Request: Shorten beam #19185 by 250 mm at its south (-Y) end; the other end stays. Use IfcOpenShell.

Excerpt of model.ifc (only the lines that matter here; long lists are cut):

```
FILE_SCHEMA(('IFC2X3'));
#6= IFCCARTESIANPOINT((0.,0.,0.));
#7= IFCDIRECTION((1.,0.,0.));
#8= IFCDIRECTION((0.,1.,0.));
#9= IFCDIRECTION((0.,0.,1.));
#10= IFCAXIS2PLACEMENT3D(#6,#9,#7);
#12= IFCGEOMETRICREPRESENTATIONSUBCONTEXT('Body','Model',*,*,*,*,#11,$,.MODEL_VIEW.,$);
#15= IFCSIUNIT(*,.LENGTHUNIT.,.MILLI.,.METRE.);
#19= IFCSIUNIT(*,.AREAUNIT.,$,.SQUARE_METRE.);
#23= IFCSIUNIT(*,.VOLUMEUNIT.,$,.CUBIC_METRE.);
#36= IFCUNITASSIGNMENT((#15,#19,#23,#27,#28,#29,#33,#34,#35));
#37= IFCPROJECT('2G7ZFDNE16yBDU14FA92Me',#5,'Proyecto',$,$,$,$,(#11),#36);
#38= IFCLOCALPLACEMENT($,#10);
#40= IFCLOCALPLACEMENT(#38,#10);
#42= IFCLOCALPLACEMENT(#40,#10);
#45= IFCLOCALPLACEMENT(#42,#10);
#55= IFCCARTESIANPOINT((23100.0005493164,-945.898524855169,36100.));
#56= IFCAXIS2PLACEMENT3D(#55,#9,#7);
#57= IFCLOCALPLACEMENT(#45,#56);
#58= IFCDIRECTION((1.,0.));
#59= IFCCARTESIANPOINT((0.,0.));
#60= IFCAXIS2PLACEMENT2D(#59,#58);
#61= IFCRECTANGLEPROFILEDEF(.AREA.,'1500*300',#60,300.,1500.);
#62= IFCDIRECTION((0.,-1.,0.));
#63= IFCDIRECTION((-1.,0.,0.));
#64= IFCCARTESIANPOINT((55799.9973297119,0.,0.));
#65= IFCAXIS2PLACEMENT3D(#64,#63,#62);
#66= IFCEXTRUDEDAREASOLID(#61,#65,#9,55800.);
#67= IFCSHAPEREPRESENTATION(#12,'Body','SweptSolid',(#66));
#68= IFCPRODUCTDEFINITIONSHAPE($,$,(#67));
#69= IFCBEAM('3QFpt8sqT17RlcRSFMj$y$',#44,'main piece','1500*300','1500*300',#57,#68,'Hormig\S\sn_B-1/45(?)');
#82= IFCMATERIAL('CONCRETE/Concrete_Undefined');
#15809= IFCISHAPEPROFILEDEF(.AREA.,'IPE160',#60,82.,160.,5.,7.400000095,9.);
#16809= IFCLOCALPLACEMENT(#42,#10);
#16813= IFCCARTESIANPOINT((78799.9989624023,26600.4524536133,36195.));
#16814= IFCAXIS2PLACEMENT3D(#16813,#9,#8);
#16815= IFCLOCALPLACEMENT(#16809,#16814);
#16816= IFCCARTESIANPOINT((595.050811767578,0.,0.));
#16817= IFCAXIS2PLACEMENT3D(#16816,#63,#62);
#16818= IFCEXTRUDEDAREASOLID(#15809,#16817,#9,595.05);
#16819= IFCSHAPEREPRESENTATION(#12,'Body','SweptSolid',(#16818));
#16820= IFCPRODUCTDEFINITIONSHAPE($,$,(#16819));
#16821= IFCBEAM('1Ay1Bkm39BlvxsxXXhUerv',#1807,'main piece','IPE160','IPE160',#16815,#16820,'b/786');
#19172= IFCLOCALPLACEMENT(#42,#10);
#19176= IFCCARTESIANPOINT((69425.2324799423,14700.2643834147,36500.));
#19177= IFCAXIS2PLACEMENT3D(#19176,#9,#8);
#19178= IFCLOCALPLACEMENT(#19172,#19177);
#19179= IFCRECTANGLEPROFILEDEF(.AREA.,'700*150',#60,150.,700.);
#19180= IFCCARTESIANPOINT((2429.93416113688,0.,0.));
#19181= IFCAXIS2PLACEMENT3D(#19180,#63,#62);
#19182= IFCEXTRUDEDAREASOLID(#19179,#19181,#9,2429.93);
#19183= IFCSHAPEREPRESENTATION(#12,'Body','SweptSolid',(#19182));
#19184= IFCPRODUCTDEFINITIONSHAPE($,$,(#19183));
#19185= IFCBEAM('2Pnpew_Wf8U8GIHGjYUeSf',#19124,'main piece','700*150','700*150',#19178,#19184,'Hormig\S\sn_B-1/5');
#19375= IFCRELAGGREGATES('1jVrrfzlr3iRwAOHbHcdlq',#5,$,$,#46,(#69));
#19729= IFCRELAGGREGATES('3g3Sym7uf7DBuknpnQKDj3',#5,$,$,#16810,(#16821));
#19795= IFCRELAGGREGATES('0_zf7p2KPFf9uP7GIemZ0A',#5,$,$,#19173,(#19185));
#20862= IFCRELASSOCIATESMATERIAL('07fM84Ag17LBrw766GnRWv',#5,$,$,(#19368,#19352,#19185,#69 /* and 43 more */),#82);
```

```python
import ifcopenshell
import ifcopenshell.util.representation
import ifcopenshell.util.unit

model = ifcopenshell.open("model.ifc")
unit_scale = ifcopenshell.util.unit.calculate_unit_scale(model)

member = model.by_guid("2Pnpew_Wf8U8GIHGjYUeSf")
change = -0.25 / unit_scale

# The extrusion runs towards the end named, so only its depth changes.
body = ifcopenshell.util.representation.get_representation(member, "Model", "Body")
solid = body.Items[0]
old_length = solid.Depth
solid.Depth += change

print(f"length {old_length:g} -> {solid.Depth:g}")

model.write("model_edited.ifc")
```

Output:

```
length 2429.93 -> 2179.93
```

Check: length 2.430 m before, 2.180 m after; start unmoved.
